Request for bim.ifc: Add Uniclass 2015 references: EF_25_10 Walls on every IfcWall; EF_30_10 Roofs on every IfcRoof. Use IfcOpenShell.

First a look at what the model holds.

```python
import ifcopenshell

model = ifcopenshell.open("bim.ifc")
print(model.schema)
print("classifications:", [c.Name for c in model.by_type("IfcClassification")])
for ifc_class in ("IfcDoor", "IfcRoof", "IfcStair", "IfcWall", "IfcWindow"):
    print(ifc_class, len(model.by_type(ifc_class)))
```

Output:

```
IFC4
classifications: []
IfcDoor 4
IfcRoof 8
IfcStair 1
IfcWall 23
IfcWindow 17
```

```python
import ifcopenshell
import ifcopenshell.api.classification

model = ifcopenshell.open("bim.ifc")

system = ifcopenshell.api.classification.add_classification(model, classification="Uniclass 2015")

codes = {
    "IfcWall": ("EF_25_10", "Walls"),
    "IfcRoof": ("EF_30_10", "Roofs"),
}
for ifc_class, (code, name) in codes.items():
    products = model.by_type(ifc_class)
    ifcopenshell.api.classification.add_reference(
        model, products=products, classification=system, identification=code, name=name
    )
    print(code, len(products))

model.write("bim-out.ifc")
```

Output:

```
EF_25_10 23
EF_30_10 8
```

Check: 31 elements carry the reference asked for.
